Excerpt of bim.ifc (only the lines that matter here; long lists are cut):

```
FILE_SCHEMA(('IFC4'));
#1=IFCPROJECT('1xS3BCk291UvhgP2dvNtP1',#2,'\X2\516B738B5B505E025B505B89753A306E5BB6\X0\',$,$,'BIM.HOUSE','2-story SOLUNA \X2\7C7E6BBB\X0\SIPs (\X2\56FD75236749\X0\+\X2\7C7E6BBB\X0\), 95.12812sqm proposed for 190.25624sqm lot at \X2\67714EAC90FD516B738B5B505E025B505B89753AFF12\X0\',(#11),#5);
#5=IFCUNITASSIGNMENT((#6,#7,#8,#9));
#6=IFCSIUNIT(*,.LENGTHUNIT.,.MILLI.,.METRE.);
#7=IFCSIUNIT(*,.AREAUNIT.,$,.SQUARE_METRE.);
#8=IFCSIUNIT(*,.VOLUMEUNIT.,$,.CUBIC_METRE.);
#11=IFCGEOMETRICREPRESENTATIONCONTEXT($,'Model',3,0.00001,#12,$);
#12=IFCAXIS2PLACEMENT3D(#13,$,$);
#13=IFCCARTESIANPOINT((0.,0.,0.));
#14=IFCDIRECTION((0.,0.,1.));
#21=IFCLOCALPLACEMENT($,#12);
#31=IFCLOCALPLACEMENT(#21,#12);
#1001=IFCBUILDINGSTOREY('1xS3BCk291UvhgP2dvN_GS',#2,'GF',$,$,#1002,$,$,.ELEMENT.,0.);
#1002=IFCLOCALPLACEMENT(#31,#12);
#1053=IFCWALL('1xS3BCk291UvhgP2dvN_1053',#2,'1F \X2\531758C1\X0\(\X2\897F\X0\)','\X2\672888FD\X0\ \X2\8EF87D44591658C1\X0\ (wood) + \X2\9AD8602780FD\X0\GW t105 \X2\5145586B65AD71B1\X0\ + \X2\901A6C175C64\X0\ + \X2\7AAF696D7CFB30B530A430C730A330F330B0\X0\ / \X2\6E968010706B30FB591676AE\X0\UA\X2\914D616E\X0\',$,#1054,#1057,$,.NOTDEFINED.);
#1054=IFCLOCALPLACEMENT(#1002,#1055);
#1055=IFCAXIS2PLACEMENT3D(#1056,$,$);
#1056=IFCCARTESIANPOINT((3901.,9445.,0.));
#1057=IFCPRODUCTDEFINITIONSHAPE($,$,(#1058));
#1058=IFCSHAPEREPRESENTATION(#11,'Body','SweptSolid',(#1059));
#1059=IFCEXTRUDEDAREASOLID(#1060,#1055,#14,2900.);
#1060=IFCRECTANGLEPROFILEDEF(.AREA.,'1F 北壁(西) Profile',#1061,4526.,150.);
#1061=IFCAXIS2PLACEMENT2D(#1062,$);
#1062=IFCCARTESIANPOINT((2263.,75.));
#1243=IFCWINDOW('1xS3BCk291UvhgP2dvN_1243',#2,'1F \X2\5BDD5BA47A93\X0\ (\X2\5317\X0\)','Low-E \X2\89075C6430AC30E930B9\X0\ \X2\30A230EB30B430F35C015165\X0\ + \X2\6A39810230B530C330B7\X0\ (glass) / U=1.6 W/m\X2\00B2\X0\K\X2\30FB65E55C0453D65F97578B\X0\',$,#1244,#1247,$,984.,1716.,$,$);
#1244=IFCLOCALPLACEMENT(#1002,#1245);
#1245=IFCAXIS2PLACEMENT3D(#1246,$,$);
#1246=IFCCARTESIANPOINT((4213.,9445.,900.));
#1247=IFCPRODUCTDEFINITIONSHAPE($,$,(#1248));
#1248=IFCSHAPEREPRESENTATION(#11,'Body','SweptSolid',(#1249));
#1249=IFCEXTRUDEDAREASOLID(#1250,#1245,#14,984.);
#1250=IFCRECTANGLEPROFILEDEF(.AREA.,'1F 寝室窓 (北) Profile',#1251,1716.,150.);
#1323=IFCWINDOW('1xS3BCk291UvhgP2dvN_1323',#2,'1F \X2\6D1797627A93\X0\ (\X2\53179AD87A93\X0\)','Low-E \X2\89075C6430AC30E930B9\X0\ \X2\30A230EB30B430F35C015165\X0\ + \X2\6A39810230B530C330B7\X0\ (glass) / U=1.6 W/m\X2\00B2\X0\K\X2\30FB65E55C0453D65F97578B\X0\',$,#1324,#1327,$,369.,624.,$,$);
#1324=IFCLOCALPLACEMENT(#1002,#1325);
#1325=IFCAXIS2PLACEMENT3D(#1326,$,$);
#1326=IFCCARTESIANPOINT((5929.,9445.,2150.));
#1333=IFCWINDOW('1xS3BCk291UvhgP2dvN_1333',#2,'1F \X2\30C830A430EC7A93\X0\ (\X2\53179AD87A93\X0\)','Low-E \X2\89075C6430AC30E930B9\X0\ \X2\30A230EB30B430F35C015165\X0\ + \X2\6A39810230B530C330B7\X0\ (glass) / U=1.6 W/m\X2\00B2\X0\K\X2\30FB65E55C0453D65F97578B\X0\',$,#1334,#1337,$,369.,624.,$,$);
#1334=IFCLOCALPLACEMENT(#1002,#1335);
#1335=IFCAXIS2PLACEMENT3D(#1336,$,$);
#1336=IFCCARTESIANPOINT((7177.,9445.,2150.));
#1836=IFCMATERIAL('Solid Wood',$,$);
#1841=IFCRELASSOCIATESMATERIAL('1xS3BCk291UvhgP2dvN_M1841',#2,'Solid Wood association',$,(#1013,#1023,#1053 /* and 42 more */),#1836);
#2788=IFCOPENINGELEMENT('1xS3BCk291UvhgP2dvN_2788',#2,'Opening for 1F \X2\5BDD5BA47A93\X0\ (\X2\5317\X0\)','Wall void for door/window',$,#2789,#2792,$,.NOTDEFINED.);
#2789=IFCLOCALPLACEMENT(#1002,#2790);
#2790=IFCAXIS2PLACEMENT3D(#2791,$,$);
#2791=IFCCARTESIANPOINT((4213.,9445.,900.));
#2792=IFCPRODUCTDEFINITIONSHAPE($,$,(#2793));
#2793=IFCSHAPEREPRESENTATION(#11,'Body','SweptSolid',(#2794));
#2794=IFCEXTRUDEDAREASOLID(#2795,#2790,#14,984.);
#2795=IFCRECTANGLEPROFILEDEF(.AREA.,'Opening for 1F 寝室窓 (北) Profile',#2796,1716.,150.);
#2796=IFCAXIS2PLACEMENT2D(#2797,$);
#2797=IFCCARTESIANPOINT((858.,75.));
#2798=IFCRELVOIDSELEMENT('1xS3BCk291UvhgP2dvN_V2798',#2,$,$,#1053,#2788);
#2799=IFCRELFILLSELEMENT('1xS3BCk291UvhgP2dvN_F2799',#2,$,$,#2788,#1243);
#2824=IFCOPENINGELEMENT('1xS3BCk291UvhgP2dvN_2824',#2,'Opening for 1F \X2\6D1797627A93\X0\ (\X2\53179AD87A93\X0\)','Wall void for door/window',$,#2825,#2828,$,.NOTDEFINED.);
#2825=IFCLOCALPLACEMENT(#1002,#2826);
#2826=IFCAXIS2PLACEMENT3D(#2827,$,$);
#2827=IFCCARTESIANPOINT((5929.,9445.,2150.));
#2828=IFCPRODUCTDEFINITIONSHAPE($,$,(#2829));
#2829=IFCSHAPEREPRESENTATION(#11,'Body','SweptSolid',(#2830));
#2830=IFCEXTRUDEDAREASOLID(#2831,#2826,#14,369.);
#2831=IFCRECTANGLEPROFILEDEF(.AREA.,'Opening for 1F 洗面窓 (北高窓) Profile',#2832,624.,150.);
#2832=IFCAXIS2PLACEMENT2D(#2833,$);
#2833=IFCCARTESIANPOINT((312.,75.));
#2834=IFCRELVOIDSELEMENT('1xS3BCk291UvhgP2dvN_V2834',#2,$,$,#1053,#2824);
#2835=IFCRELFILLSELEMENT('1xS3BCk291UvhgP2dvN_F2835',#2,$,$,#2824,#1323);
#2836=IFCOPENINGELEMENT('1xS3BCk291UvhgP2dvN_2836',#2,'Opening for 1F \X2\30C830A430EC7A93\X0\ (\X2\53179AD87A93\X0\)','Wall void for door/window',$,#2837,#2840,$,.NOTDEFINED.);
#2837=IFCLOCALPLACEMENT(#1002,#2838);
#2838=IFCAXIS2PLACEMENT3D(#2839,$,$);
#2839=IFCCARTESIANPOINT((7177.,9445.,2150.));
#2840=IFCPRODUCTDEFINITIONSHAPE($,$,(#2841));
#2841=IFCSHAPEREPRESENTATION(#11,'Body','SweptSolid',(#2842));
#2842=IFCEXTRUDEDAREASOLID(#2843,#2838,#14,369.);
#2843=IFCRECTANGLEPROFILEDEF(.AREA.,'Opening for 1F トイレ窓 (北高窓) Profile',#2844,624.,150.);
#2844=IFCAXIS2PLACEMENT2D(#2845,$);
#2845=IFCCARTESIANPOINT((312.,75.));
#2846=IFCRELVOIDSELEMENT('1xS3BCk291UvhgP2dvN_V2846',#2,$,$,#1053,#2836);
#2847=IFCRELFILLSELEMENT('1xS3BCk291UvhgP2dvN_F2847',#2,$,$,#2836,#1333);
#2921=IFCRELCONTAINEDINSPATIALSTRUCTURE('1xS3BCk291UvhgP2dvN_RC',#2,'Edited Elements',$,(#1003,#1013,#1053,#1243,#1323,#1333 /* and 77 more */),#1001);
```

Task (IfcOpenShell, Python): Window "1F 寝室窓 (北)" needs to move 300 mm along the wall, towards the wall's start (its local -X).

```python
import ifcopenshell
import ifcopenshell.api.geometry
import ifcopenshell.util.placement
import ifcopenshell.util.unit

model = ifcopenshell.open("bim.ifc")
unit_scale = ifcopenshell.util.unit.calculate_unit_scale(model)

window = model.by_guid("1xS3BCk291UvhgP2dvN_1243")
opening = window.FillsVoids[0].RelatingOpeningElement
wall = opening.VoidsElements[0].RelatingBuildingElement

wall_matrix = ifcopenshell.util.placement.get_local_placement(wall.ObjectPlacement)
shift = wall_matrix[:3, 0] * -0.3 / unit_scale
before = ifcopenshell.util.placement.get_local_placement(window.ObjectPlacement)[:3, 3].copy()

# The window is not placed relative to its opening, so move both.
for product in (opening, window):
    matrix = ifcopenshell.util.placement.get_local_placement(product.ObjectPlacement)
    matrix[:3, 3] += shift
    ifcopenshell.api.geometry.edit_object_placement(model, product=product, matrix=matrix, is_si=False)

after = ifcopenshell.util.placement.get_local_placement(window.ObjectPlacement)[:3, 3]
print("window moved by", (after - before).round(3) + 0.0)

model.write("bim_v2.ifc")
```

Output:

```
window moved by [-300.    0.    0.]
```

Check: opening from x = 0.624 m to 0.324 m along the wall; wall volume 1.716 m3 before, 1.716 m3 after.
